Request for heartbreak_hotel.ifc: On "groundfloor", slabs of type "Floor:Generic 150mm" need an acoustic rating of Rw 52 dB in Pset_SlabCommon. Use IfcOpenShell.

First a look at what the model holds.

```python
import ifcopenshell
import ifcopenshell.util.element

model = ifcopenshell.open("heartbreak_hotel.ifc")
print(model.schema)
storey = next(s for s in model.by_type("IfcBuildingStorey") if s.Name == "groundfloor")
slabs = [e for e in ifcopenshell.util.element.get_decomposition(storey) if e.is_a("IfcSlab")]
seen = {}
for e in slabs:
    element_type = ifcopenshell.util.element.get_type(e)
    key = (element_type.Name if element_type != e and element_type else None, ifcopenshell.util.element.get_pset(e, "Pset_SlabCommon", "AcousticRating"))
    seen[key] = seen.get(key, 0) + 1
for (name, value), count in sorted(seen.items(), key=str):
    print(count, "x", name, "|", value)
```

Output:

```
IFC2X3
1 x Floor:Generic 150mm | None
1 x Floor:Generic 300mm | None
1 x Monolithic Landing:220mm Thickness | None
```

```python
import ifcopenshell
import ifcopenshell.api.pset
import ifcopenshell.util.element

model = ifcopenshell.open("heartbreak_hotel.ifc")

storey = next(s for s in model.by_type("IfcBuildingStorey") if s.Name == "groundfloor")
slabs = [e for e in ifcopenshell.util.element.get_decomposition(storey) if e.is_a("IfcSlab")]

count = 0
for e in slabs:
    element_type = ifcopenshell.util.element.get_type(e)
    if element_type in (None, e) or element_type.Name != "Floor:Generic 150mm":
        continue
    # add_pset returns the element's existing set when there is one.
    pset = ifcopenshell.api.pset.add_pset(model, product=e, name="Pset_SlabCommon")
    ifcopenshell.api.pset.edit_pset(model, pset=pset, properties={"AcousticRating": "Rw 52 dB"})
    count += 1

print(count, "slabs updated")

model.write("heartbreak_hotel-out.ifc")
```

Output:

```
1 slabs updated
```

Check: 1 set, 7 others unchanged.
